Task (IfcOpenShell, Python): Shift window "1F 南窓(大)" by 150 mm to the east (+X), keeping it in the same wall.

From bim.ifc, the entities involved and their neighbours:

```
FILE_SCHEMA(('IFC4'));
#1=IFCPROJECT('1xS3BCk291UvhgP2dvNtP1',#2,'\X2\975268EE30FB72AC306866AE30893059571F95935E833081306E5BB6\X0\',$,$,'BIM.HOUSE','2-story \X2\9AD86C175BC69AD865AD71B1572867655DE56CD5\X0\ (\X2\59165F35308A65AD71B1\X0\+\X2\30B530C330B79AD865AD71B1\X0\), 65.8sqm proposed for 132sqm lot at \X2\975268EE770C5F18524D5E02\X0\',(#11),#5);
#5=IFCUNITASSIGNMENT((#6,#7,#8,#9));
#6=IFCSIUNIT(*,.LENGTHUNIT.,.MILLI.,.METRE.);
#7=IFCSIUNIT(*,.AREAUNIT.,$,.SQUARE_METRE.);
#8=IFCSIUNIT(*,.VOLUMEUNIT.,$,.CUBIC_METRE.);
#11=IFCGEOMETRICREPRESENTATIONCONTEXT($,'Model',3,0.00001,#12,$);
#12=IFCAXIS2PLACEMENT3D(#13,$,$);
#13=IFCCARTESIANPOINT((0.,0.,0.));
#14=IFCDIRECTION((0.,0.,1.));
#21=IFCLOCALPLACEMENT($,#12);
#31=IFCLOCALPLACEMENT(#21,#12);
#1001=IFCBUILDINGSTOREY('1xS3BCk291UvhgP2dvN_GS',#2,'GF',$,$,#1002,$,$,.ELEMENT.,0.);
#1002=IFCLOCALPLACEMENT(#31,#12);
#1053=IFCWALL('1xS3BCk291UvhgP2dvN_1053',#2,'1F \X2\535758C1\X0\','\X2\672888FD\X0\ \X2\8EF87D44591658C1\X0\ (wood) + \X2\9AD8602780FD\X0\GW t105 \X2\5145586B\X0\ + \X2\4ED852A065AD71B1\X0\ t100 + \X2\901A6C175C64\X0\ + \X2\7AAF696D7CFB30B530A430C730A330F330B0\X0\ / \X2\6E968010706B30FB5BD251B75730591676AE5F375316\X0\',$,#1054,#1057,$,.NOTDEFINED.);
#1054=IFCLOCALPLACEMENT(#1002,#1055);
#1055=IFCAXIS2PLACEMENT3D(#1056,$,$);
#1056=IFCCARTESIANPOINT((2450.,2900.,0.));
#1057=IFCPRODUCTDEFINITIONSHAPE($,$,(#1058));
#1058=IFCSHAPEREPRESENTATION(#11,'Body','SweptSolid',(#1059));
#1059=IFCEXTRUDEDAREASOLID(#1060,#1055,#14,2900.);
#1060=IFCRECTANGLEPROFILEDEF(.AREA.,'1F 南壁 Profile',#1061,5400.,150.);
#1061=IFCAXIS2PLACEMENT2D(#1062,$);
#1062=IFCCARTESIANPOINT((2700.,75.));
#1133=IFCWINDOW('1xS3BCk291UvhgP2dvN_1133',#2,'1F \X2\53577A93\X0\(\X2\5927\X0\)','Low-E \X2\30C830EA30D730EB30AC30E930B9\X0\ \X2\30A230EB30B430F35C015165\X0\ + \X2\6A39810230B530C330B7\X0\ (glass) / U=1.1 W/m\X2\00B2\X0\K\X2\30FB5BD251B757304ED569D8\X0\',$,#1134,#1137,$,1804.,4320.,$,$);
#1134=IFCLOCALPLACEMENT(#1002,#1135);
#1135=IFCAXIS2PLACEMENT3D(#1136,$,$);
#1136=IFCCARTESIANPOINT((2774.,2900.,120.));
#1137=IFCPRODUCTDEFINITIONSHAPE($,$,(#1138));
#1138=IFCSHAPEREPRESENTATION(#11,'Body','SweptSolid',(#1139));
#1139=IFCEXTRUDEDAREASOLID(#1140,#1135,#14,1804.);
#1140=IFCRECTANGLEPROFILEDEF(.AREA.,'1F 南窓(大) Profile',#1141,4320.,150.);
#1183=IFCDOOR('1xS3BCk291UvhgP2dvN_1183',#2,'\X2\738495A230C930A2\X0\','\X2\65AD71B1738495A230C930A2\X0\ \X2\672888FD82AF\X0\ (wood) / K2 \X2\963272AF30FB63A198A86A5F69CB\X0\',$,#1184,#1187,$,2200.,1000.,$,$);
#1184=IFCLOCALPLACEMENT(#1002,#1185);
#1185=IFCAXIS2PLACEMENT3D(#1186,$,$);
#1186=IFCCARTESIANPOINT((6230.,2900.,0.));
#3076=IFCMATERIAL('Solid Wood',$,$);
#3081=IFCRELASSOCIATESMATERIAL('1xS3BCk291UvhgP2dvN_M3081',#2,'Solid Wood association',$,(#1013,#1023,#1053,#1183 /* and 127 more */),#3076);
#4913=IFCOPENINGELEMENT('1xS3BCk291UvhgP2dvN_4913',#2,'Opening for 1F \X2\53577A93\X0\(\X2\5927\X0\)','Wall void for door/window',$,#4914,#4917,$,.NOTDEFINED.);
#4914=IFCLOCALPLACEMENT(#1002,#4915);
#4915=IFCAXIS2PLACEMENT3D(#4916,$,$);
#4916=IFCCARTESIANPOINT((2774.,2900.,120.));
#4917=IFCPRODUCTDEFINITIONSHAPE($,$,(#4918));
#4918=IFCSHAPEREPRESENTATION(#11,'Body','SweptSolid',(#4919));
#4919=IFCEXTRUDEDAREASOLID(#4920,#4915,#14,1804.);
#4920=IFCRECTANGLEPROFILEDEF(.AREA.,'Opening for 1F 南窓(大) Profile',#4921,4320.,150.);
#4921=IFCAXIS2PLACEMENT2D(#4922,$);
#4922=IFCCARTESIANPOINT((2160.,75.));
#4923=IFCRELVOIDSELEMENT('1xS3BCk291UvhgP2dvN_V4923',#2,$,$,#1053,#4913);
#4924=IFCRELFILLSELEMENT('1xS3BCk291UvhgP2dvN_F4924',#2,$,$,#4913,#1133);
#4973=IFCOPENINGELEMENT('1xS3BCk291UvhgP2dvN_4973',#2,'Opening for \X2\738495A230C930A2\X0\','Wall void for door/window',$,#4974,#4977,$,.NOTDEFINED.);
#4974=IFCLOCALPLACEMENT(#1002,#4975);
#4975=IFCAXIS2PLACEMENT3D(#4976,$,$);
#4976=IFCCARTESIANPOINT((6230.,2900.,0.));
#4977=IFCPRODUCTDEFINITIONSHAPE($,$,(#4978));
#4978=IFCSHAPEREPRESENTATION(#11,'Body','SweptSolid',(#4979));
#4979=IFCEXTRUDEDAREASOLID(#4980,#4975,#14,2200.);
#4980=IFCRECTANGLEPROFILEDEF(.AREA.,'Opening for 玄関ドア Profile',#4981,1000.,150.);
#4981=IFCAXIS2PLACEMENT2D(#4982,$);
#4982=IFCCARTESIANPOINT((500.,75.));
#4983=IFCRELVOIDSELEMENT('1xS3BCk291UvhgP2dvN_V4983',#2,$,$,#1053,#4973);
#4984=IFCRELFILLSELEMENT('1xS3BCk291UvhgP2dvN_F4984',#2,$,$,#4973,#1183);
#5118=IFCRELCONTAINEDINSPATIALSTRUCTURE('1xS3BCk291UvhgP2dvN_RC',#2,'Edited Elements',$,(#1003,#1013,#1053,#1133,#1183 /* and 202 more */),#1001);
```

```python
import ifcopenshell
import ifcopenshell.api.geometry
import ifcopenshell.util.placement
import ifcopenshell.util.unit

model = ifcopenshell.open("bim.ifc")
unit_scale = ifcopenshell.util.unit.calculate_unit_scale(model)

window = model.by_guid("1xS3BCk291UvhgP2dvN_1133")
opening = window.FillsVoids[0].RelatingOpeningElement
wall = opening.VoidsElements[0].RelatingBuildingElement

wall_matrix = ifcopenshell.util.placement.get_local_placement(wall.ObjectPlacement)
shift = wall_matrix[:3, 0] * 0.15 / unit_scale
before = ifcopenshell.util.placement.get_local_placement(window.ObjectPlacement)[:3, 3].copy()

# The window is not placed relative to its opening, so move both.
for product in (opening, window):
    matrix = ifcopenshell.util.placement.get_local_placement(product.ObjectPlacement)
    matrix[:3, 3] += shift
    ifcopenshell.api.geometry.edit_object_placement(model, product=product, matrix=matrix, is_si=False)

after = ifcopenshell.util.placement.get_local_placement(window.ObjectPlacement)[:3, 3]
print("window moved by", (after - before).round(3) + 0.0)

model.write("bim_rev.ifc")
```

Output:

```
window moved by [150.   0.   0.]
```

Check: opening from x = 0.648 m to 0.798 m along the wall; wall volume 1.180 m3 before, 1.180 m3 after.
